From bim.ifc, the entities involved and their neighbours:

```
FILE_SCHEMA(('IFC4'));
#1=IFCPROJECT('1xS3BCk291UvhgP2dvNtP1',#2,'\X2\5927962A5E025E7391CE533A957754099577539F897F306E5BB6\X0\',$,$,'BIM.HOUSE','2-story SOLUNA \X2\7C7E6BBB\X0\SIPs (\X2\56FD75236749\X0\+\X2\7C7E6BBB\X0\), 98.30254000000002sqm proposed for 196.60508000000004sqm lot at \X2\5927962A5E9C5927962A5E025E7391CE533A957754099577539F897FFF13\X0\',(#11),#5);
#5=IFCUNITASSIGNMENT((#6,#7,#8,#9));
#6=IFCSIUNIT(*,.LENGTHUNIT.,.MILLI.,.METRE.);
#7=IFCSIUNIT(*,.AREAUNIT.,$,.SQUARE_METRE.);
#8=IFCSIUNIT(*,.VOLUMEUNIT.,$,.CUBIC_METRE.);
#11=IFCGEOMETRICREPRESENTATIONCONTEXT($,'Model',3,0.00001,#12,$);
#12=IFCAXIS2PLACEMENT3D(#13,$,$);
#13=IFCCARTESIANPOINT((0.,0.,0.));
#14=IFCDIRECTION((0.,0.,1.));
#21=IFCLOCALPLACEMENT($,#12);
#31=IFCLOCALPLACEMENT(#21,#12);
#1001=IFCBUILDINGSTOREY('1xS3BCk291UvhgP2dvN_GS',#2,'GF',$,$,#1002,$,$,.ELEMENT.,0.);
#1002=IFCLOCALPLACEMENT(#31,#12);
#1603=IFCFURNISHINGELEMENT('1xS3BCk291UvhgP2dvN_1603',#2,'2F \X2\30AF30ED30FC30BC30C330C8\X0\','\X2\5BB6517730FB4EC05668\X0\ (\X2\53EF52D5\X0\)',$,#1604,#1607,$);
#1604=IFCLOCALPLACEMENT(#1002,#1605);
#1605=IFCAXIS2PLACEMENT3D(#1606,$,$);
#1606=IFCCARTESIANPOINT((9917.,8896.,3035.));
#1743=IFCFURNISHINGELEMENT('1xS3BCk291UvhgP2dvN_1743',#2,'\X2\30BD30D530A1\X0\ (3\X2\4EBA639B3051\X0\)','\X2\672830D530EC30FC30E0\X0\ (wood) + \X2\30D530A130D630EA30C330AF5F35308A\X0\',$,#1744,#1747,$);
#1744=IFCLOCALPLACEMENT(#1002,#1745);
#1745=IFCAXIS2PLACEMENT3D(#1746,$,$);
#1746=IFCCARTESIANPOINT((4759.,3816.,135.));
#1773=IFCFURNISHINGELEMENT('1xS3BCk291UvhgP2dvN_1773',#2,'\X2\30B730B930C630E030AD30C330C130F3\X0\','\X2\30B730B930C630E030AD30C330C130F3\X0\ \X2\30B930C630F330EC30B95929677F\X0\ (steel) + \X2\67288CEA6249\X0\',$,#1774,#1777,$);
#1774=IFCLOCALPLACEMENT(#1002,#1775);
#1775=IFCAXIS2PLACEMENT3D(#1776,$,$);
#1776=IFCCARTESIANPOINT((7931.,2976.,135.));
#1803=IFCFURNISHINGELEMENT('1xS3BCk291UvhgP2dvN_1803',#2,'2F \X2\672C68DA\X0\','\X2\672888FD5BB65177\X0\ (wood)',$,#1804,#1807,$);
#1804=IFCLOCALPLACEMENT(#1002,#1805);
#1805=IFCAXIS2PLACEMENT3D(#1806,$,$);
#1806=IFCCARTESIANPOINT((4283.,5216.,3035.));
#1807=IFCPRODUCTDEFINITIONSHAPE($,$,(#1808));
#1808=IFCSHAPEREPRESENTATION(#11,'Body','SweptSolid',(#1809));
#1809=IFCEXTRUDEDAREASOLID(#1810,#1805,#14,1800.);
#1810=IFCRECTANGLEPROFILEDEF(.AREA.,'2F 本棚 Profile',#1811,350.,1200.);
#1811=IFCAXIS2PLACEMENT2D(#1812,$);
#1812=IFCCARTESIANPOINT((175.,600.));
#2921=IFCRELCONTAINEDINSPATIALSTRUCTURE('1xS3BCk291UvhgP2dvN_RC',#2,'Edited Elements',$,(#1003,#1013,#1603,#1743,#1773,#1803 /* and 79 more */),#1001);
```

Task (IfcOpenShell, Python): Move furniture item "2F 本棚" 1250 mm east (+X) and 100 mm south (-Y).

```python
import ifcopenshell
import ifcopenshell.api.geometry
import ifcopenshell.util.placement

model = ifcopenshell.open("bim.ifc")

item = model.by_id(1803)
matrix = ifcopenshell.util.placement.get_local_placement(item.ObjectPlacement)
matrix[0, 3] += 1250.0
matrix[1, 3] -= 100.0
ifcopenshell.api.geometry.edit_object_placement(model, product=item, matrix=matrix, is_si=False)

print(ifcopenshell.util.placement.get_local_placement(item.ObjectPlacement).round(3) + 0.0)

model.write("bim_v2.ifc")
```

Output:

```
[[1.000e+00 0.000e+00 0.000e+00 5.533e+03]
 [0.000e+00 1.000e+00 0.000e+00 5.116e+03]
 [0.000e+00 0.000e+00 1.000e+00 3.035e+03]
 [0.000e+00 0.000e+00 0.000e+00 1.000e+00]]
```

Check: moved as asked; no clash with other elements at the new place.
